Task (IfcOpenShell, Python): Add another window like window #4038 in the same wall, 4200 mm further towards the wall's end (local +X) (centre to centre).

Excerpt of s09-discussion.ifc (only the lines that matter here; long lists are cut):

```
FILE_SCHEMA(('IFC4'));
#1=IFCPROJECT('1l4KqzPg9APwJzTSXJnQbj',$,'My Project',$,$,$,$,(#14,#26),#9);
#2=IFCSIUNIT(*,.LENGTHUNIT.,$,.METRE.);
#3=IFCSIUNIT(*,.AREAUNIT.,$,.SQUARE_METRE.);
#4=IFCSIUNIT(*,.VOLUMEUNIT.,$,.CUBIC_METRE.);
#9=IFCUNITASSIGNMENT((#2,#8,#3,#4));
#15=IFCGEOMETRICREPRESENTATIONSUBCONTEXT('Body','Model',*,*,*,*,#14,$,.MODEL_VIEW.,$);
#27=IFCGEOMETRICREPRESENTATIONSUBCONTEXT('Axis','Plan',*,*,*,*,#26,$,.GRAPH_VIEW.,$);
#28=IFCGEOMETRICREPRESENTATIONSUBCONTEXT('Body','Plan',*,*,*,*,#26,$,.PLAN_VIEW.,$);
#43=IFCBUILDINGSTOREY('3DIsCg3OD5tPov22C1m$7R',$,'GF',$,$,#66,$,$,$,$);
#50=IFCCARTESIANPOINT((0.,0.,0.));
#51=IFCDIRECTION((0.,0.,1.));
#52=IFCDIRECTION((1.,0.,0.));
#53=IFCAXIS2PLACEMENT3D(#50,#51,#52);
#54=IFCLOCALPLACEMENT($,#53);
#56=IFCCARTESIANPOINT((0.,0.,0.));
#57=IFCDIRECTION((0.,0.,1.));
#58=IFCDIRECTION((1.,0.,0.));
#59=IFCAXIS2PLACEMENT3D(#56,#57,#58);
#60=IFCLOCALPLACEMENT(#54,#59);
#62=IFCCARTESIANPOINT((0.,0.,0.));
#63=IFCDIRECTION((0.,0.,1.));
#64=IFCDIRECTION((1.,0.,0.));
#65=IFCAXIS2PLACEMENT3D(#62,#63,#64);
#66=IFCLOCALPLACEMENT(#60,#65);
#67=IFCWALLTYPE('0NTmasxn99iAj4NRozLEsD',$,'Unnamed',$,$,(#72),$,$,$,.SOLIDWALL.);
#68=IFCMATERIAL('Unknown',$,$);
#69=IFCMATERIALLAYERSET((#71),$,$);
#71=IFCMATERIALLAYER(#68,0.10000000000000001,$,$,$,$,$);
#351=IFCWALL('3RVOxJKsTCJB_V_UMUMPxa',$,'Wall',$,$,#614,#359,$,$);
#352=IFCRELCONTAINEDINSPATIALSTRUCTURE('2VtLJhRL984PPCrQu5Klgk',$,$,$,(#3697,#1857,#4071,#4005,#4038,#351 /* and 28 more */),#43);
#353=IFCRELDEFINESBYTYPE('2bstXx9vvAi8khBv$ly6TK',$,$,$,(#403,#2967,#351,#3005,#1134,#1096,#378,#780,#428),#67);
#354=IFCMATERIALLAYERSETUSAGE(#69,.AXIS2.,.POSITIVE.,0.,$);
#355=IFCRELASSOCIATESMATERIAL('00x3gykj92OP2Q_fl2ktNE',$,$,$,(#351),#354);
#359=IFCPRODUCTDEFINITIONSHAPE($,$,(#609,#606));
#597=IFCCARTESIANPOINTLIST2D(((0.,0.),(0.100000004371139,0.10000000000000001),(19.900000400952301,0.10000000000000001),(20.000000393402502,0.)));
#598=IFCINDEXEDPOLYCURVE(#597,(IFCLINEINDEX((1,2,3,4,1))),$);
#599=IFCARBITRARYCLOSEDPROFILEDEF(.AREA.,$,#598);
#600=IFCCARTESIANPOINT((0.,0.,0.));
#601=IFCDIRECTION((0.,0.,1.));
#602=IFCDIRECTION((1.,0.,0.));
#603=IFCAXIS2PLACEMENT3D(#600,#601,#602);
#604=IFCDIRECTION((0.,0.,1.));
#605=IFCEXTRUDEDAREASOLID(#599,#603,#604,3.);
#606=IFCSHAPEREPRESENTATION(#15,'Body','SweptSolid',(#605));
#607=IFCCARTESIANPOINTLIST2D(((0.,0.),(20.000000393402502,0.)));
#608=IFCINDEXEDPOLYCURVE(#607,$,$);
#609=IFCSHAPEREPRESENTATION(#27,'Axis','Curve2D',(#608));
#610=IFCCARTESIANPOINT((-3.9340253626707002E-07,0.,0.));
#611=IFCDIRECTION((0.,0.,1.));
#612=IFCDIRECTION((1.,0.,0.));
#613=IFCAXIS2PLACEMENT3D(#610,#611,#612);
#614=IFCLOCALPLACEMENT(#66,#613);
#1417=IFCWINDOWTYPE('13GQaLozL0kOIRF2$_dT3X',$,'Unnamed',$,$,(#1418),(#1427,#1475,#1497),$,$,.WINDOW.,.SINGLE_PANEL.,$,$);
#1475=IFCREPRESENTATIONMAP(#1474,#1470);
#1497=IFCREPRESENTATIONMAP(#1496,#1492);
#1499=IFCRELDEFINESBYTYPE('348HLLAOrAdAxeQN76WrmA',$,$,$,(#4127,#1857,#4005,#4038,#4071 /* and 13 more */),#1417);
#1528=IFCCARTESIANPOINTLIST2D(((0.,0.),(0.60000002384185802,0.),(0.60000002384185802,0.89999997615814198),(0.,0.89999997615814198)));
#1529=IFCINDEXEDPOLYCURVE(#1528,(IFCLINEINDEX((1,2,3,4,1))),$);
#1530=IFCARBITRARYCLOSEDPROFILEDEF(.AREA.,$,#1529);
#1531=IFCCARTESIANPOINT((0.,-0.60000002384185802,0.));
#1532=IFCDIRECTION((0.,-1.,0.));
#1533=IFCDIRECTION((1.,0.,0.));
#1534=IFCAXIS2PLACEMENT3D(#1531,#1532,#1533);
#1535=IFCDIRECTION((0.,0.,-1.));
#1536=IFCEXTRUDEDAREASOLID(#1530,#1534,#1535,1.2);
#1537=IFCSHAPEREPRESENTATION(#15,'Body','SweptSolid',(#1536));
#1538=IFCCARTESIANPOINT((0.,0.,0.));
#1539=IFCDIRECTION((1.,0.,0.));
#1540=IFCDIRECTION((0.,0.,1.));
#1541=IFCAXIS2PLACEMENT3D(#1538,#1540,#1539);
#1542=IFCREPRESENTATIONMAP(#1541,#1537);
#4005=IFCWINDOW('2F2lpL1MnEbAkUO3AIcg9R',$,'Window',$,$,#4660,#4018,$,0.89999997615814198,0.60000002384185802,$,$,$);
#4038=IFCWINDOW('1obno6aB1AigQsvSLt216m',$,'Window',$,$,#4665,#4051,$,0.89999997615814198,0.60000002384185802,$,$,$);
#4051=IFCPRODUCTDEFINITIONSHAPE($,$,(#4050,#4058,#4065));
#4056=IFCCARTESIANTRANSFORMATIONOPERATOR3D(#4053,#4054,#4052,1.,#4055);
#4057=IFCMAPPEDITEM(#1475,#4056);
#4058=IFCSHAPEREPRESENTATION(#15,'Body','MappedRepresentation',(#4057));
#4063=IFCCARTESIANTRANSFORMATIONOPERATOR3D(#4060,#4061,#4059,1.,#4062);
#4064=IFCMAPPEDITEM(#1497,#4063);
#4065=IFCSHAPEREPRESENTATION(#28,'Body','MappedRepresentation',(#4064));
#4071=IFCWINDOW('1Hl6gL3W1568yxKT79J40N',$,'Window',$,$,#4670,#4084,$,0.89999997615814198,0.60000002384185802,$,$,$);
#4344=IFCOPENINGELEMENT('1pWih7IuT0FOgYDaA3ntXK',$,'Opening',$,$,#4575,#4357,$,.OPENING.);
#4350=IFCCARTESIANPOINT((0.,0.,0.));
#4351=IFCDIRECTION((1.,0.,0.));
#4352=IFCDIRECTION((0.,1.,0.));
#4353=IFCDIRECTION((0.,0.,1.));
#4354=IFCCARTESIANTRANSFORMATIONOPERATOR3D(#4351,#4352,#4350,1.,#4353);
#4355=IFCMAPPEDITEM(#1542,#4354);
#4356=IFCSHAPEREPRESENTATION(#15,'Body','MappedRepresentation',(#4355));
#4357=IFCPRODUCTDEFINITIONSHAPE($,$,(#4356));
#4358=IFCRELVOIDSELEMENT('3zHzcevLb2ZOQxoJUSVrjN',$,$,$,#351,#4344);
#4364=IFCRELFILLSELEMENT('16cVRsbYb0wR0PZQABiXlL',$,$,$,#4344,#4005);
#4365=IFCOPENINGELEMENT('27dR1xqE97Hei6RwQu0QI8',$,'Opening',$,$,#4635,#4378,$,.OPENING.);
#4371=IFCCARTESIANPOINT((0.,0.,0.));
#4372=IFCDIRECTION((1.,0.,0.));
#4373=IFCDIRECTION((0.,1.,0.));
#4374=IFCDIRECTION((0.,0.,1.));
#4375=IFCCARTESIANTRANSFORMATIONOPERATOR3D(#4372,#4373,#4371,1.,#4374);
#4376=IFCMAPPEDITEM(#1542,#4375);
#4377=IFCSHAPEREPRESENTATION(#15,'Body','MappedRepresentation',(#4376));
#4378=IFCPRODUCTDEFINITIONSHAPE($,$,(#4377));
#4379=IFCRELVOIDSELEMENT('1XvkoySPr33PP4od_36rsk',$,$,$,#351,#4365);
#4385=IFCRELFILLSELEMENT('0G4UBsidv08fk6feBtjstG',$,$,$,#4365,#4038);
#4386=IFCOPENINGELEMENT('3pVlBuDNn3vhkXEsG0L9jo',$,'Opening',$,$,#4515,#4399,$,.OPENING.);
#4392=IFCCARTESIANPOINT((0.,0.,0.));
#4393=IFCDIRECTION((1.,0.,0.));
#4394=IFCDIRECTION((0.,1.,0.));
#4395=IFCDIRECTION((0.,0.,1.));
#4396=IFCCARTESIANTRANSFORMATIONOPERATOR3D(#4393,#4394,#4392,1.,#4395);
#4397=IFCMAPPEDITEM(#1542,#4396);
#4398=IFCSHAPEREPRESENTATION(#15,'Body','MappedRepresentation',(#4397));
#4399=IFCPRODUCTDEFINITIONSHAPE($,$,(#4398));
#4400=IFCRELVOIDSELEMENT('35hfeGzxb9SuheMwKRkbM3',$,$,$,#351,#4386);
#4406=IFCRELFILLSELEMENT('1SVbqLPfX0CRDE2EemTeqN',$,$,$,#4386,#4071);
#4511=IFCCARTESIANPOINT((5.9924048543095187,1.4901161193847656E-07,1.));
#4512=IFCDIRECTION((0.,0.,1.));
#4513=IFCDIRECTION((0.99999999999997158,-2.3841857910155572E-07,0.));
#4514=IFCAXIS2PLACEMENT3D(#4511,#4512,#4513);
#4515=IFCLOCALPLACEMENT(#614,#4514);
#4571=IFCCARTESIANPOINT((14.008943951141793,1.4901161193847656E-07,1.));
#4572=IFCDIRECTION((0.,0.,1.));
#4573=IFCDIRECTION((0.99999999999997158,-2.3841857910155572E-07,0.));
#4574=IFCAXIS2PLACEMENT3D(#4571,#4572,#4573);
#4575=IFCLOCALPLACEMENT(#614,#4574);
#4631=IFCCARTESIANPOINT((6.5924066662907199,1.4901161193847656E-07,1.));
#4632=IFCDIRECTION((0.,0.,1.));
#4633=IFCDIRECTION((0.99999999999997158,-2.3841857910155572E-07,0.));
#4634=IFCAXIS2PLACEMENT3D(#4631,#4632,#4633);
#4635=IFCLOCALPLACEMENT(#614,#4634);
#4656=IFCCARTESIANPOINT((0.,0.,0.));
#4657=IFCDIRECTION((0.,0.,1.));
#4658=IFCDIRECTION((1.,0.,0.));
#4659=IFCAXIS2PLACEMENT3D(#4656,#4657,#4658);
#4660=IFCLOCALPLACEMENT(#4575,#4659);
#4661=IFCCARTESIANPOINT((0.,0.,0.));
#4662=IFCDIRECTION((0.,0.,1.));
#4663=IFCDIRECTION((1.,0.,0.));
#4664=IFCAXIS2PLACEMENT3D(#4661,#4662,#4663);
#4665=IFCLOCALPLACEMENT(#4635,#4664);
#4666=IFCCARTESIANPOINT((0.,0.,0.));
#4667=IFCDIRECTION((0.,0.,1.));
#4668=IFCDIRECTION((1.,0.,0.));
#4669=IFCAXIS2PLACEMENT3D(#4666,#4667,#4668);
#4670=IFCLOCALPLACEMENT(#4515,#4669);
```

```python
import ifcopenshell
import ifcopenshell.api.feature
import ifcopenshell.api.geometry
import ifcopenshell.api.root
import ifcopenshell.geom
import ifcopenshell.util.element
import ifcopenshell.util.placement
import ifcopenshell.util.shape
import ifcopenshell.util.unit

model = ifcopenshell.open("s09-discussion.ifc")
unit_scale = ifcopenshell.util.unit.calculate_unit_scale(model)
settings = ifcopenshell.geom.settings()


def volume(element):
    """Net volume in cubic metres, openings subtracted."""
    shape = ifcopenshell.geom.create_shape(settings, element)
    return ifcopenshell.util.shape.get_volume(shape.geometry)


window = model.by_guid("1obno6aB1AigQsvSLt216m")
opening = window.FillsVoids[0].RelatingOpeningElement
wall = opening.VoidsElements[0].RelatingBuildingElement
before = volume(wall)
shift = ifcopenshell.util.placement.get_local_placement(wall.ObjectPlacement)[:3, 0] * 4.2 / unit_scale

# copy_class copies the void relationship, type, container and properties, but no geometry.
new_opening = ifcopenshell.api.root.copy_class(model, product=opening)
new_opening.Representation = ifcopenshell.util.element.copy_deep(
    model, opening.Representation, exclude=["IfcGeometricRepresentationContext", "IfcRepresentationMap"]
)
new_window = ifcopenshell.api.root.copy_class(model, product=window)
new_window.Representation = ifcopenshell.util.element.copy_deep(
    model, window.Representation, exclude=["IfcGeometricRepresentationContext", "IfcRepresentationMap"]
)
ifcopenshell.api.feature.add_filling(model, opening=new_opening, element=new_window)

for old, new in ((opening, new_opening), (window, new_window)):
    matrix = ifcopenshell.util.placement.get_local_placement(old.ObjectPlacement)
    matrix[:3, 3] += shift
    ifcopenshell.api.geometry.edit_object_placement(model, product=new, matrix=matrix, is_si=False)

after = volume(wall)

print(f"wall volume {before:.3f} -> {after:.3f} m3")

model.write("s09-discussion-out.ifc")
```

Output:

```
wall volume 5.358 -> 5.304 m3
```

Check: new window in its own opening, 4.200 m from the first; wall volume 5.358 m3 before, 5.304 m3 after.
